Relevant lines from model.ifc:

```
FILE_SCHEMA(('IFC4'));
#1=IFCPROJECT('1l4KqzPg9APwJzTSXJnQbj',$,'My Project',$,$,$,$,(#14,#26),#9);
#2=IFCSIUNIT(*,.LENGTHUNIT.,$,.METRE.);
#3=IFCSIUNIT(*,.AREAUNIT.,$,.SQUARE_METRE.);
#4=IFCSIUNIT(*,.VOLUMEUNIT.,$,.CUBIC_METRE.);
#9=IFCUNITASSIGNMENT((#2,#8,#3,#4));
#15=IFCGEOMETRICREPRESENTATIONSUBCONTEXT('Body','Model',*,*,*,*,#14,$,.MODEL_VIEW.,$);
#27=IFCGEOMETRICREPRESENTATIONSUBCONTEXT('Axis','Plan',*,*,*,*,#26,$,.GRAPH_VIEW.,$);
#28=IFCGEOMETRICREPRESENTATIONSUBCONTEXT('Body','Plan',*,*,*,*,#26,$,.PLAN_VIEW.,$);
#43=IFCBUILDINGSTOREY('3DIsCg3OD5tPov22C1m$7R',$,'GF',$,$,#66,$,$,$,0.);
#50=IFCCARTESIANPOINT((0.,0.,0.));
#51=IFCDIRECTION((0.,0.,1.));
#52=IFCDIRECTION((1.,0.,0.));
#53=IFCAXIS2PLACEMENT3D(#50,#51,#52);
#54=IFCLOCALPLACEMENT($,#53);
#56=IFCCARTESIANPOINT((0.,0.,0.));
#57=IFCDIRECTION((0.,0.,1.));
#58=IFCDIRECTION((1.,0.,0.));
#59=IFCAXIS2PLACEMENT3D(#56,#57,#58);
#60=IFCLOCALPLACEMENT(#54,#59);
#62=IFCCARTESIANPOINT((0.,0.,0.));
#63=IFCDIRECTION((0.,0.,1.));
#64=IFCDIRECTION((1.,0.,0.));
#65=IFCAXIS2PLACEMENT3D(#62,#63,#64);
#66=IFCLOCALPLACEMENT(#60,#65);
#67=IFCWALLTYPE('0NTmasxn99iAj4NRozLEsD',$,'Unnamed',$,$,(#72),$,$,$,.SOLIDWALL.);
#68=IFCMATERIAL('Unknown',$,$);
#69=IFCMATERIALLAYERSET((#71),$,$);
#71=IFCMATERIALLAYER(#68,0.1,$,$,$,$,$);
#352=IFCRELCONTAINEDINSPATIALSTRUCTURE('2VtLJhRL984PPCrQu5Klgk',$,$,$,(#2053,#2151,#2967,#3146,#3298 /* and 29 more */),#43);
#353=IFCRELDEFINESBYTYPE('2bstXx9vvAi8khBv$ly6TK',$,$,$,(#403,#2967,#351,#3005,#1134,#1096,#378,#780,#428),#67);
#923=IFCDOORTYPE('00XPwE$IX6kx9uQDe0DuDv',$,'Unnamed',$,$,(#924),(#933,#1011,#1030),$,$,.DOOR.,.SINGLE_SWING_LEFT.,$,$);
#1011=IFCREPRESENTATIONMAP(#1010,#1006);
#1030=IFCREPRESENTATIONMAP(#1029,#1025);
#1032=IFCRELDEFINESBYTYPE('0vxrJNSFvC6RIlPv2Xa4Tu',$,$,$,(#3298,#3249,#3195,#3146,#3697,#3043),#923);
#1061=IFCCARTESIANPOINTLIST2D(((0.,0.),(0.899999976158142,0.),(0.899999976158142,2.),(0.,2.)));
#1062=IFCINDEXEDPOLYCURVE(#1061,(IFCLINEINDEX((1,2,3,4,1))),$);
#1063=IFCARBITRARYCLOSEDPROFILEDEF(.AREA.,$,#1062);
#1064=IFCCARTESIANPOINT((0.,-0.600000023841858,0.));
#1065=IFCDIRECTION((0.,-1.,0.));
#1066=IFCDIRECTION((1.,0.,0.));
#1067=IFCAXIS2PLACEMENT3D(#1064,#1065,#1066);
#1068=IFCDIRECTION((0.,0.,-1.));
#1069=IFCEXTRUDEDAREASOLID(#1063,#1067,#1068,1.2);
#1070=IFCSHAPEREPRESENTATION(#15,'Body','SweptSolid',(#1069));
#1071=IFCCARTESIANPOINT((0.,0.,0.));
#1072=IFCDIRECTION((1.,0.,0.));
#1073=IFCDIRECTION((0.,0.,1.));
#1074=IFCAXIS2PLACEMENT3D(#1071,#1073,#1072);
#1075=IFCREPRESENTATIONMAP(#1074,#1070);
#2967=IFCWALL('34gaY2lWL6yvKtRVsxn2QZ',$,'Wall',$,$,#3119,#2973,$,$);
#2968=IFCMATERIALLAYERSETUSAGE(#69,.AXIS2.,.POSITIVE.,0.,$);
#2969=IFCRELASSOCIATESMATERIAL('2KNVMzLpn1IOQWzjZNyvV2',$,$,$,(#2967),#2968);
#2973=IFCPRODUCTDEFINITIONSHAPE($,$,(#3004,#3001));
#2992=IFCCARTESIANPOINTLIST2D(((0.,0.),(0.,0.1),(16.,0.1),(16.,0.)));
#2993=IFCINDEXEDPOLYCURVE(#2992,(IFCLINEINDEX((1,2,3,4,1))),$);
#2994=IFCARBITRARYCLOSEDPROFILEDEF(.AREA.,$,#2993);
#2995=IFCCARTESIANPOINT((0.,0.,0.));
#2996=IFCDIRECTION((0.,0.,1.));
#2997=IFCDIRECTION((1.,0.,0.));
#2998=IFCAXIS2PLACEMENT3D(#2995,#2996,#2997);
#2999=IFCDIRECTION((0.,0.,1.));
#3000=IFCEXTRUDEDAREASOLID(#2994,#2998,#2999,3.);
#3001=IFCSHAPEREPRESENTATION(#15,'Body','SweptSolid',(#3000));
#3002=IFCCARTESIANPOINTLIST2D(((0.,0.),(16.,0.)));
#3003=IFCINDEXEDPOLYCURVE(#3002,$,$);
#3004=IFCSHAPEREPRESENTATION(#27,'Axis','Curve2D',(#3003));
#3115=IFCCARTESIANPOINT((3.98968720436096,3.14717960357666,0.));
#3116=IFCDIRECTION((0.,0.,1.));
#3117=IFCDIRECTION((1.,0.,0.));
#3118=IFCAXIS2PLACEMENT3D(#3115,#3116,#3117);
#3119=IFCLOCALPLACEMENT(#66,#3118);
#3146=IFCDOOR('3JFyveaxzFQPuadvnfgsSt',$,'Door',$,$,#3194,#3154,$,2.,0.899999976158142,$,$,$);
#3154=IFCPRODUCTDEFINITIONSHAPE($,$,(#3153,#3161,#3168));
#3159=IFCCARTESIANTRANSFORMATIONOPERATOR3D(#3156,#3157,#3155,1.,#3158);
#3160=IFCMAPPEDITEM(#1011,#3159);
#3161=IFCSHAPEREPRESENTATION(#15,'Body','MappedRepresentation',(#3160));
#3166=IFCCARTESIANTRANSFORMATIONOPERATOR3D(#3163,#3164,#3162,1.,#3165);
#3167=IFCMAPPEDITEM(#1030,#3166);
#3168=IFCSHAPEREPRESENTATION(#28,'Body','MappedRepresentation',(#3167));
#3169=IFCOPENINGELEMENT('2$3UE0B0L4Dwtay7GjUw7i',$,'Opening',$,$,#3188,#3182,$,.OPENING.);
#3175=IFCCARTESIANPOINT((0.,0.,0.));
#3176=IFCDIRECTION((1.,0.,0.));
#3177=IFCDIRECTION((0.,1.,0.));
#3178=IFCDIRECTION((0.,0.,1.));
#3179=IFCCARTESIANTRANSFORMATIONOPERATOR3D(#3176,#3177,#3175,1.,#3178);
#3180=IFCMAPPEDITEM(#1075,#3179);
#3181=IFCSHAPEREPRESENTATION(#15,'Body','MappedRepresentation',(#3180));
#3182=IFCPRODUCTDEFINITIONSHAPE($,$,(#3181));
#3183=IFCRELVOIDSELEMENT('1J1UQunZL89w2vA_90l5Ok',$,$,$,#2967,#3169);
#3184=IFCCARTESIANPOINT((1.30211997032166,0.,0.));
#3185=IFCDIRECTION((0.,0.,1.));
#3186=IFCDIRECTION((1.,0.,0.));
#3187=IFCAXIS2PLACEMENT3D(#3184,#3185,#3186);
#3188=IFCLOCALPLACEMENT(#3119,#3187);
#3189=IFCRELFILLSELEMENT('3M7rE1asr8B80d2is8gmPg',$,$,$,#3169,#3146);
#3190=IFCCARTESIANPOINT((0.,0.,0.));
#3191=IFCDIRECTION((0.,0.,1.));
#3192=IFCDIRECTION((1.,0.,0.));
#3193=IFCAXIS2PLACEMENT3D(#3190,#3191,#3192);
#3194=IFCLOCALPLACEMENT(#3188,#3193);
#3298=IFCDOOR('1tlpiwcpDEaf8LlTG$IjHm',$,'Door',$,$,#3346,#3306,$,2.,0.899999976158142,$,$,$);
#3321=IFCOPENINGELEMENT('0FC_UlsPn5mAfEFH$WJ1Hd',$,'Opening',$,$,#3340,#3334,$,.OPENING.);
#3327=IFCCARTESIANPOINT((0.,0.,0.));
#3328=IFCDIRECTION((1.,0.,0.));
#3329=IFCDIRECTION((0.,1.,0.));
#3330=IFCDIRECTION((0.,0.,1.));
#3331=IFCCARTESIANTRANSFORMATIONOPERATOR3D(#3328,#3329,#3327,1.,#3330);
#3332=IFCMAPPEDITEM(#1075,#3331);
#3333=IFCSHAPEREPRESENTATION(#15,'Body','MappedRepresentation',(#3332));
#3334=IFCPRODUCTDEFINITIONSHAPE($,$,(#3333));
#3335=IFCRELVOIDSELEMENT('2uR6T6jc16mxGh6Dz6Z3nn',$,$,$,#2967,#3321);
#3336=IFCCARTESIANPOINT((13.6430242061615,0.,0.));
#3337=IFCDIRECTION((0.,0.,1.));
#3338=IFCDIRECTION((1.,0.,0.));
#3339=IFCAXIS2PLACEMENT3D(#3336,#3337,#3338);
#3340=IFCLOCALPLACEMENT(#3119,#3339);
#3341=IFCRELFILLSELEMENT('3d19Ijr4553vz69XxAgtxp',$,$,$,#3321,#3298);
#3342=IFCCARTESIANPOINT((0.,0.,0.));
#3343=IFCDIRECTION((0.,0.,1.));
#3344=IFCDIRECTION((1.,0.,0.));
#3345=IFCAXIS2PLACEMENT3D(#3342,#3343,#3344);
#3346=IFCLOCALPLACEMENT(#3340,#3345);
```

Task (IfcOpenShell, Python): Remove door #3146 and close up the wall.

```python
import ifcopenshell
import ifcopenshell.api.feature
import ifcopenshell.api.root
import ifcopenshell.geom
import ifcopenshell.util.shape

model = ifcopenshell.open("model.ifc")
settings = ifcopenshell.geom.settings()


def volume(element):
    """Net volume in cubic metres, openings subtracted."""
    shape = ifcopenshell.geom.create_shape(settings, element)
    return ifcopenshell.util.shape.get_volume(shape.geometry)


door = model.by_guid("3JFyveaxzFQPuadvnfgsSt")
opening = door.FillsVoids[0].RelatingOpeningElement
wall = opening.VoidsElements[0].RelatingBuildingElement
before = volume(wall)

ifcopenshell.api.root.remove_product(model, product=door)
ifcopenshell.api.feature.remove_feature(model, feature=opening)

after = volume(wall)

print(f"wall volume {before:.3f} -> {after:.3f} m3")

model.write("model_updated.ifc")
```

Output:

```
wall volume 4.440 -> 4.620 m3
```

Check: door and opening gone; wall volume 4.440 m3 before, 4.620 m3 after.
